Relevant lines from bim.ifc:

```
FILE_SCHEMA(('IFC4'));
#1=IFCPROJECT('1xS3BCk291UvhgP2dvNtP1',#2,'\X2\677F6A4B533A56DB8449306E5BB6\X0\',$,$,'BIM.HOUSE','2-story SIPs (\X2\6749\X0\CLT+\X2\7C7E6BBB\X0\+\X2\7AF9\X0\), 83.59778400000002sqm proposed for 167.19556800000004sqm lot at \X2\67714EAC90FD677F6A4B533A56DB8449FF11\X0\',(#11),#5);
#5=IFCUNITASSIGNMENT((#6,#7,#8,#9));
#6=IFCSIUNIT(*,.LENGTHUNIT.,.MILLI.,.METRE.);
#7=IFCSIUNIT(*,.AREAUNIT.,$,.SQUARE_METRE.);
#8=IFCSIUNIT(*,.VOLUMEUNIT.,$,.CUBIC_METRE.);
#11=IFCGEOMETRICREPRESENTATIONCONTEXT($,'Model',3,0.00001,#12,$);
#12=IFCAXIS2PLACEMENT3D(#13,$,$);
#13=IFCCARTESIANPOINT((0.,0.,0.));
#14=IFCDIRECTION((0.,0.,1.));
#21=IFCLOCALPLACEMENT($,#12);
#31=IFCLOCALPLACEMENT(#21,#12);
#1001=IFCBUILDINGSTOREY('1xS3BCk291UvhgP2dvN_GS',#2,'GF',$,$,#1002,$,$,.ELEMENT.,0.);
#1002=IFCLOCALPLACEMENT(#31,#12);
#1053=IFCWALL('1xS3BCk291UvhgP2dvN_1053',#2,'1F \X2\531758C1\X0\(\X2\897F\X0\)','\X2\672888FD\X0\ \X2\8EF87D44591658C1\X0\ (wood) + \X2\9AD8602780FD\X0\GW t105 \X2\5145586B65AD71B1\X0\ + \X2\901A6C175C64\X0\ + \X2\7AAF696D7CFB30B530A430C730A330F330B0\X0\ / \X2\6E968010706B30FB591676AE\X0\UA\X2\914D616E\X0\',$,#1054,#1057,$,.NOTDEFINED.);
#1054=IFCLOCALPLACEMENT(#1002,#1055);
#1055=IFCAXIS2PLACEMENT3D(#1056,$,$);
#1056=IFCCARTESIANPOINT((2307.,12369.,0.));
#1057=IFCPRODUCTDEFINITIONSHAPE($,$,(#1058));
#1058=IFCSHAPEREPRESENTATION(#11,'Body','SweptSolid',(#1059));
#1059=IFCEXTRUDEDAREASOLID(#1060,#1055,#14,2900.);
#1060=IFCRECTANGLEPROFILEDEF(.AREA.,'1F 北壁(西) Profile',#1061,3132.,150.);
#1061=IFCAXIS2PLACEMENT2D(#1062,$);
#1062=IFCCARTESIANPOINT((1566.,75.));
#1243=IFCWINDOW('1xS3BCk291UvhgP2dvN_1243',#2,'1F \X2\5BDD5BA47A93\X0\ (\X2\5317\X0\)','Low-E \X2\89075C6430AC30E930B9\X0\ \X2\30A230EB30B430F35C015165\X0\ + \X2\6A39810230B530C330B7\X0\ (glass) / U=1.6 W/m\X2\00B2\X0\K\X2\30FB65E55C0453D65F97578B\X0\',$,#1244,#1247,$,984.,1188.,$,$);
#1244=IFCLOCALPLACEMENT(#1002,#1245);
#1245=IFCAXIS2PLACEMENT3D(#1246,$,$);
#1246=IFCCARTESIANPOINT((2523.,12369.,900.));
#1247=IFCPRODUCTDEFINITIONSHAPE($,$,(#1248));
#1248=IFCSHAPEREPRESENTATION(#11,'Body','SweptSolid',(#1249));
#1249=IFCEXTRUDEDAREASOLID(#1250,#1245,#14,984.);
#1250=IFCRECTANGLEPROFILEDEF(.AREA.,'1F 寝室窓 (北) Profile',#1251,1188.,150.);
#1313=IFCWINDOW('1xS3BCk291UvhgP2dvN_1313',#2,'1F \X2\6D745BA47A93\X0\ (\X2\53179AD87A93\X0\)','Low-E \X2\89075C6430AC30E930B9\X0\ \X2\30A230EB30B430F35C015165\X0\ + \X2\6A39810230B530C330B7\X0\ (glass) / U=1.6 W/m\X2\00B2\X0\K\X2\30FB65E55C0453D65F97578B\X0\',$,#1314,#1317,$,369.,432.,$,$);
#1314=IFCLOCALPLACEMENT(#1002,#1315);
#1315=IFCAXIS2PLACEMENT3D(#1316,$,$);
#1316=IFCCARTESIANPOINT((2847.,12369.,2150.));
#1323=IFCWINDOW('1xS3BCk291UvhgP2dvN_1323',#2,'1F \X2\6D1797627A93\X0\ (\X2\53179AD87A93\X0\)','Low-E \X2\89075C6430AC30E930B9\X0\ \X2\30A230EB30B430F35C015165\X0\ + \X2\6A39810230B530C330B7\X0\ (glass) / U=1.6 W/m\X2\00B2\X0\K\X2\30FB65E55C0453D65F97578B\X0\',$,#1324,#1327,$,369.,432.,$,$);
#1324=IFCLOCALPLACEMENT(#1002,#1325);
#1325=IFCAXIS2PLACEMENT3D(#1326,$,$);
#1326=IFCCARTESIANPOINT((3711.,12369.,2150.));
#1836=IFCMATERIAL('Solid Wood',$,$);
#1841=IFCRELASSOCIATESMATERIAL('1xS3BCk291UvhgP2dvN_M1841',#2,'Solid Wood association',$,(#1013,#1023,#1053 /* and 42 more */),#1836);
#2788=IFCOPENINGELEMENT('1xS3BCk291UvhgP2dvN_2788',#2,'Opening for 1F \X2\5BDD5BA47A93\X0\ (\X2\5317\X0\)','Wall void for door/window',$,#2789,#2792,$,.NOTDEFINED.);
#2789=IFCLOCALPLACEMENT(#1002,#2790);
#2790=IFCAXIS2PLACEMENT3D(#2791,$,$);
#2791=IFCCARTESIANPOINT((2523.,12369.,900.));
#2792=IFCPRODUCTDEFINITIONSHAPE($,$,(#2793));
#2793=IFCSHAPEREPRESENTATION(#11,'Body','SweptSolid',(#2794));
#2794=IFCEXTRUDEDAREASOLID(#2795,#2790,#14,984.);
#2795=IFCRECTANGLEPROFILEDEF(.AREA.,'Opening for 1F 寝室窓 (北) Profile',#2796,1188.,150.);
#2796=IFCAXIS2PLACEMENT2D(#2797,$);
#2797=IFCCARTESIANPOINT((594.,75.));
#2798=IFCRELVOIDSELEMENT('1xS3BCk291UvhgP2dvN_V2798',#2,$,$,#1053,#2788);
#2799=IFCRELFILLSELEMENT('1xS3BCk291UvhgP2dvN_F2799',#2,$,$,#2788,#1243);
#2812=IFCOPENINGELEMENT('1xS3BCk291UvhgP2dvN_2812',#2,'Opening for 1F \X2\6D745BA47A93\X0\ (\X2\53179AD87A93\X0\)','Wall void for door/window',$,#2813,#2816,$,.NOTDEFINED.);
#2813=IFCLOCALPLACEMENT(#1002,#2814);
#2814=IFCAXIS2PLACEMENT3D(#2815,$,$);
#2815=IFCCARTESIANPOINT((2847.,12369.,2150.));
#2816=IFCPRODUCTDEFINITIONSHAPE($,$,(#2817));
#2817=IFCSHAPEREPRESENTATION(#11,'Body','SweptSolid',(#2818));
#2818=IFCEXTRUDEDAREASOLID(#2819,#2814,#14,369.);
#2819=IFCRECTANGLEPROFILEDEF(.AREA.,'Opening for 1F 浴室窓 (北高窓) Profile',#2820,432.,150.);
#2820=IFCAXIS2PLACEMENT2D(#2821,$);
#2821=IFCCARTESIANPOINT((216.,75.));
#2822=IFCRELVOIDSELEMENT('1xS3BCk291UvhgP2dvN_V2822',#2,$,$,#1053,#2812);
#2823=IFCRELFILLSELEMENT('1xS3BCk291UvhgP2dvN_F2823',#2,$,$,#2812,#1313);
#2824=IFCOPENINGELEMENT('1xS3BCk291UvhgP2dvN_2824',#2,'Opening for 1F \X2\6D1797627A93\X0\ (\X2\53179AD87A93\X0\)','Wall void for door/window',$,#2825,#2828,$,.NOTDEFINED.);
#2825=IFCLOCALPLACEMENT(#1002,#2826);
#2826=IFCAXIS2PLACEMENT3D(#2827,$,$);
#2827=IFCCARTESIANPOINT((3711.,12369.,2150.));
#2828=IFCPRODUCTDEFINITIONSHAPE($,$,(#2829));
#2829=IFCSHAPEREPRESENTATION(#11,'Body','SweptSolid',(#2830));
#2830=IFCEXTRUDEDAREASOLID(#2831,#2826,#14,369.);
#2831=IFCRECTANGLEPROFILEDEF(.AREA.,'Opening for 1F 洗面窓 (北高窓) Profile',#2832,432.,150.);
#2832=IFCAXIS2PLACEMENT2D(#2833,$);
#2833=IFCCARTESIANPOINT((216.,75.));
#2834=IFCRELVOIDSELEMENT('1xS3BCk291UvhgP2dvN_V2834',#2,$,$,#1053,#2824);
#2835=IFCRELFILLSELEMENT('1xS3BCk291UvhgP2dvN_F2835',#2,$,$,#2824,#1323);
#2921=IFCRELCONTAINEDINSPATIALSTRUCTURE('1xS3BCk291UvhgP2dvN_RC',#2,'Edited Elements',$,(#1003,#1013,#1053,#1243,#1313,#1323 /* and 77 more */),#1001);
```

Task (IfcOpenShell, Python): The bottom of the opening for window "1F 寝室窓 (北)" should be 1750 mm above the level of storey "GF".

```python
import numpy as np
import ifcopenshell
import ifcopenshell.api.geometry
import ifcopenshell.geom
import ifcopenshell.util.element
import ifcopenshell.util.placement
import ifcopenshell.util.shape
import ifcopenshell.util.unit

model = ifcopenshell.open("bim.ifc")
unit_scale = ifcopenshell.util.unit.calculate_unit_scale(model)

window = model.by_id(1243)
opening = window.FillsVoids[0].RelatingOpeningElement
storey = ifcopenshell.util.element.get_container(window, ifc_class="IfcBuildingStorey")
level = ifcopenshell.util.placement.get_local_placement(storey.ObjectPlacement)[2, 3]

# The opening's origin need not be at the sill, so measure its lowest point.
shape = ifcopenshell.geom.create_shape(ifcopenshell.geom.settings(), opening)
bottom = ifcopenshell.util.shape.get_shape_bottom_elevation(shape, shape.geometry) / unit_scale
dz = level + 1.75 / unit_scale - bottom

shift = np.array([0.0, 0.0, dz])
# The window is not placed relative to its opening, so move both.
for product in (opening, window):
    matrix = ifcopenshell.util.placement.get_local_placement(product.ObjectPlacement)
    matrix[:3, 3] += shift
    ifcopenshell.api.geometry.edit_object_placement(model, product=product, matrix=matrix, is_si=False)

print(f"moved by {dz * unit_scale:+.3f} m")

model.write("bim_updated.ifc")
```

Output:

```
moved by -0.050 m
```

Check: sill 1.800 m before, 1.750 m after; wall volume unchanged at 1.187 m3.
